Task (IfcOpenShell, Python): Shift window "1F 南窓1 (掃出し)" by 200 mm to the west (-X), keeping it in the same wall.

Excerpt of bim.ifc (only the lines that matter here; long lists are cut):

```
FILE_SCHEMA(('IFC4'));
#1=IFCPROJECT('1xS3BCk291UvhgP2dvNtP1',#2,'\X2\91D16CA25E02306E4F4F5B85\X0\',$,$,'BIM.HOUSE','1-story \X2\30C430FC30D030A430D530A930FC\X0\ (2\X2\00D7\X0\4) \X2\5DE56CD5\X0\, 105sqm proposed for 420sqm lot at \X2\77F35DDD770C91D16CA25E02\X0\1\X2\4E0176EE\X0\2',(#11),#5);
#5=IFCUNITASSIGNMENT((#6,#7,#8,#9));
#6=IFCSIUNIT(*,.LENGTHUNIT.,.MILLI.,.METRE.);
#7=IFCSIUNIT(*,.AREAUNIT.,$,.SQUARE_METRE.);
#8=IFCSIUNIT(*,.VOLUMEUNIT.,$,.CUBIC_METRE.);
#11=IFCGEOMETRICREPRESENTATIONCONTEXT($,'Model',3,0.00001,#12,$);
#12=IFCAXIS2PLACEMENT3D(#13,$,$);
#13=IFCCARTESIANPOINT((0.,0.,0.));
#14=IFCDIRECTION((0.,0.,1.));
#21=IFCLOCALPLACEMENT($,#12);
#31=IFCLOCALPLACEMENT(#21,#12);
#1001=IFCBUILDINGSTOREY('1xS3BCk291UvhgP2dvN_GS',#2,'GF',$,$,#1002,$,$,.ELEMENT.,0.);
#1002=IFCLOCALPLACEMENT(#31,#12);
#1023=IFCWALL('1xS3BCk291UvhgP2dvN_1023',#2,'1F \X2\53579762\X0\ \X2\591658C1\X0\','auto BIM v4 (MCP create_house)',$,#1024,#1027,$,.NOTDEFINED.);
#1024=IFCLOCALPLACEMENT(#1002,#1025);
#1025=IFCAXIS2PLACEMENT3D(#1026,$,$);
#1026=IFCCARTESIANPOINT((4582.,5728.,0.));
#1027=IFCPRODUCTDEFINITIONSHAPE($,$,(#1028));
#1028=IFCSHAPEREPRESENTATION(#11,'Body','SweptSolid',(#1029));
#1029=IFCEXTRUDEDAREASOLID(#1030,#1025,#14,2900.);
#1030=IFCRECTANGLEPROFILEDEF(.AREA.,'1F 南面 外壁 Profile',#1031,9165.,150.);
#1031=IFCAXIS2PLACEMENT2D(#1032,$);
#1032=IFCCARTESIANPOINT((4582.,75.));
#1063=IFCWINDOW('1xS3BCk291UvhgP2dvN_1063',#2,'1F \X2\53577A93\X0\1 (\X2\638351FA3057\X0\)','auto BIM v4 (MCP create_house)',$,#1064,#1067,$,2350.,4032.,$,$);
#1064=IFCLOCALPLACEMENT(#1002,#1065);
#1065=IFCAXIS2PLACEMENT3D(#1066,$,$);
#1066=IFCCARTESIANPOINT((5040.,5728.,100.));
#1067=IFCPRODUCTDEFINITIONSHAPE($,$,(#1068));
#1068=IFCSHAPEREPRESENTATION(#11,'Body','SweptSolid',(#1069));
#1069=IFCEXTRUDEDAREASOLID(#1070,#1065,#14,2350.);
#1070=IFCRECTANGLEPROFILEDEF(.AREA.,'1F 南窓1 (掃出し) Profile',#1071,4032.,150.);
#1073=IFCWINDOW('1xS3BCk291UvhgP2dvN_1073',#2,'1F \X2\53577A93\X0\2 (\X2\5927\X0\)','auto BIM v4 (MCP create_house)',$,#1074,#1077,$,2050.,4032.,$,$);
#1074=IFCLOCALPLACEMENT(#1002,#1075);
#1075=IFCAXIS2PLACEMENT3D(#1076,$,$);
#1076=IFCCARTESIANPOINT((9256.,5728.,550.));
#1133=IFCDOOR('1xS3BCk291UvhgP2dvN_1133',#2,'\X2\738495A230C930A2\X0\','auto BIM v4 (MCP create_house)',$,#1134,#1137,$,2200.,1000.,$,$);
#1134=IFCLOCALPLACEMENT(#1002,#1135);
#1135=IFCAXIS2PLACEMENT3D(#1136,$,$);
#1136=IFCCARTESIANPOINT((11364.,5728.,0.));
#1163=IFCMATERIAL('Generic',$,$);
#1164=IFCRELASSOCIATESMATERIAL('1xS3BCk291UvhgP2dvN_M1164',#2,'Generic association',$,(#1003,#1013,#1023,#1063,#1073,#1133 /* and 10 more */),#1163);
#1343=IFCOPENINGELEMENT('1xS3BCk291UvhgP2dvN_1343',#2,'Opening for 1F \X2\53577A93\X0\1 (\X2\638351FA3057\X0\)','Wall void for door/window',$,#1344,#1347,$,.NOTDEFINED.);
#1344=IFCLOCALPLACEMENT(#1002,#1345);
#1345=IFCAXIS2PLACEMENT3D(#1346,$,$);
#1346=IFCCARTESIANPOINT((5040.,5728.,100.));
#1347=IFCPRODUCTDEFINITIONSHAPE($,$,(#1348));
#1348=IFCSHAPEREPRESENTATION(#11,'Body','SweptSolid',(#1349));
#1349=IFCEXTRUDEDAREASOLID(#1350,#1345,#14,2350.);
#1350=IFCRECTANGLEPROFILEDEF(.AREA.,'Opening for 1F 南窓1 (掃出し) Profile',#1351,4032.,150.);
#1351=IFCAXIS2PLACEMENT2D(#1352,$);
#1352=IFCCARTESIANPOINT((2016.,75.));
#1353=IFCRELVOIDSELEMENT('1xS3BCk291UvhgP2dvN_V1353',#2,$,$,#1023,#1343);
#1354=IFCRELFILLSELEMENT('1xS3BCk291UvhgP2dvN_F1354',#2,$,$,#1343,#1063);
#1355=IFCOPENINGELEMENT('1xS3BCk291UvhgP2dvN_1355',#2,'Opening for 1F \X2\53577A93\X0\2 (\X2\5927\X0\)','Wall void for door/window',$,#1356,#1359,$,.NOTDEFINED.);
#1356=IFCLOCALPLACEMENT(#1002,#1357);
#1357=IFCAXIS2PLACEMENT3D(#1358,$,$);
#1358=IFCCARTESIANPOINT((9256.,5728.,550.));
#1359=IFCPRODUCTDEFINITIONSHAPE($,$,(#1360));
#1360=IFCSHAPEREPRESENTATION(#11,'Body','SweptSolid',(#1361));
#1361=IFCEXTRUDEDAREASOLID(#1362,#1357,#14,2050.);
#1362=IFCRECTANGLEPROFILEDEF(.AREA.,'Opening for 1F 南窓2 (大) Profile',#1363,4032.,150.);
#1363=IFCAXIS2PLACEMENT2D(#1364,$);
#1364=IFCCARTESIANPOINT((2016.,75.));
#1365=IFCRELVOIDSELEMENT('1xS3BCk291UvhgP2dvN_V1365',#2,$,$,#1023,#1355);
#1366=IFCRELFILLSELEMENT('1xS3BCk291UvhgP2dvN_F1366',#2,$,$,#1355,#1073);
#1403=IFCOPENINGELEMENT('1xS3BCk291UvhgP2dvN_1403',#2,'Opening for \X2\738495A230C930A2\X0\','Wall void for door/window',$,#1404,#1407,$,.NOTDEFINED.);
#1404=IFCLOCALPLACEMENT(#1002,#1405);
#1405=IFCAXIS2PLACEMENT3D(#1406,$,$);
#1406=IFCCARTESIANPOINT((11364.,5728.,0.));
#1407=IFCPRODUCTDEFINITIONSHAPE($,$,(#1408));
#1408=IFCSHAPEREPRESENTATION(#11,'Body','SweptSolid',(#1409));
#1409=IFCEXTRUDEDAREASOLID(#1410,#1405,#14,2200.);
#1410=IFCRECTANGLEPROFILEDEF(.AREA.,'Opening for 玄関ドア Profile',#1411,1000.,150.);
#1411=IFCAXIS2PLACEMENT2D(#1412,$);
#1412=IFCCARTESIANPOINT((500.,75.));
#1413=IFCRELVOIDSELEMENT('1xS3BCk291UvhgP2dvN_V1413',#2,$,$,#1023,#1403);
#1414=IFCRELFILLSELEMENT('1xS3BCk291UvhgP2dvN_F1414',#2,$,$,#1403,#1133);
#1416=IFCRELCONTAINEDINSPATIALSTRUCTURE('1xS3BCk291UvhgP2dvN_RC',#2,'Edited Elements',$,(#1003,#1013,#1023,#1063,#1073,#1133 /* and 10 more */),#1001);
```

```python
import ifcopenshell
import ifcopenshell.api.geometry
import ifcopenshell.util.placement
import ifcopenshell.util.unit

model = ifcopenshell.open("bim.ifc")
unit_scale = ifcopenshell.util.unit.calculate_unit_scale(model)

window = model.by_guid("1xS3BCk291UvhgP2dvN_1063")
opening = window.FillsVoids[0].RelatingOpeningElement
wall = opening.VoidsElements[0].RelatingBuildingElement

wall_matrix = ifcopenshell.util.placement.get_local_placement(wall.ObjectPlacement)
shift = wall_matrix[:3, 0] * -0.2 / unit_scale
before = ifcopenshell.util.placement.get_local_placement(window.ObjectPlacement)[:3, 3].copy()

# The window is not placed relative to its opening, so move both.
for product in (opening, window):
    matrix = ifcopenshell.util.placement.get_local_placement(product.ObjectPlacement)
    matrix[:3, 3] += shift
    ifcopenshell.api.geometry.edit_object_placement(model, product=product, matrix=matrix, is_si=False)

after = ifcopenshell.util.placement.get_local_placement(window.ObjectPlacement)[:3, 3]
print("window moved by", (after - before).round(3) + 0.0)

model.write("bim-out.ifc")
```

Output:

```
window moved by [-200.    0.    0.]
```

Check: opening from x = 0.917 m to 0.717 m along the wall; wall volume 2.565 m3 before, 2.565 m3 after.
